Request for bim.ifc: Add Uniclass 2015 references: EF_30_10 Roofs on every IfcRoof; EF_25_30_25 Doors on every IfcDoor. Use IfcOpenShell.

First a look at what the model holds.

```python
import ifcopenshell

model = ifcopenshell.open("bim.ifc")
print(model.schema)
print("classifications:", [c.Name for c in model.by_type("IfcClassification")])
for ifc_class in ("IfcDoor", "IfcRoof", "IfcStair", "IfcWall", "IfcWindow"):
    print(ifc_class, len(model.by_type(ifc_class)))
```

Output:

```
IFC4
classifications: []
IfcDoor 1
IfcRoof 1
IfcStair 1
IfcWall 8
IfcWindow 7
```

```python
import ifcopenshell
import ifcopenshell.api.classification

model = ifcopenshell.open("bim.ifc")

system = ifcopenshell.api.classification.add_classification(model, classification="Uniclass 2015")

codes = {
    "IfcRoof": ("EF_30_10", "Roofs"),
    "IfcDoor": ("EF_25_30_25", "Doors"),
}
for ifc_class, (code, name) in codes.items():
    products = model.by_type(ifc_class)
    ifcopenshell.api.classification.add_reference(
        model, products=products, classification=system, identification=code, name=name
    )
    print(code, len(products))

model.write("bim_edited.ifc")
```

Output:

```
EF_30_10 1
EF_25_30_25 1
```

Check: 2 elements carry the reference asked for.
